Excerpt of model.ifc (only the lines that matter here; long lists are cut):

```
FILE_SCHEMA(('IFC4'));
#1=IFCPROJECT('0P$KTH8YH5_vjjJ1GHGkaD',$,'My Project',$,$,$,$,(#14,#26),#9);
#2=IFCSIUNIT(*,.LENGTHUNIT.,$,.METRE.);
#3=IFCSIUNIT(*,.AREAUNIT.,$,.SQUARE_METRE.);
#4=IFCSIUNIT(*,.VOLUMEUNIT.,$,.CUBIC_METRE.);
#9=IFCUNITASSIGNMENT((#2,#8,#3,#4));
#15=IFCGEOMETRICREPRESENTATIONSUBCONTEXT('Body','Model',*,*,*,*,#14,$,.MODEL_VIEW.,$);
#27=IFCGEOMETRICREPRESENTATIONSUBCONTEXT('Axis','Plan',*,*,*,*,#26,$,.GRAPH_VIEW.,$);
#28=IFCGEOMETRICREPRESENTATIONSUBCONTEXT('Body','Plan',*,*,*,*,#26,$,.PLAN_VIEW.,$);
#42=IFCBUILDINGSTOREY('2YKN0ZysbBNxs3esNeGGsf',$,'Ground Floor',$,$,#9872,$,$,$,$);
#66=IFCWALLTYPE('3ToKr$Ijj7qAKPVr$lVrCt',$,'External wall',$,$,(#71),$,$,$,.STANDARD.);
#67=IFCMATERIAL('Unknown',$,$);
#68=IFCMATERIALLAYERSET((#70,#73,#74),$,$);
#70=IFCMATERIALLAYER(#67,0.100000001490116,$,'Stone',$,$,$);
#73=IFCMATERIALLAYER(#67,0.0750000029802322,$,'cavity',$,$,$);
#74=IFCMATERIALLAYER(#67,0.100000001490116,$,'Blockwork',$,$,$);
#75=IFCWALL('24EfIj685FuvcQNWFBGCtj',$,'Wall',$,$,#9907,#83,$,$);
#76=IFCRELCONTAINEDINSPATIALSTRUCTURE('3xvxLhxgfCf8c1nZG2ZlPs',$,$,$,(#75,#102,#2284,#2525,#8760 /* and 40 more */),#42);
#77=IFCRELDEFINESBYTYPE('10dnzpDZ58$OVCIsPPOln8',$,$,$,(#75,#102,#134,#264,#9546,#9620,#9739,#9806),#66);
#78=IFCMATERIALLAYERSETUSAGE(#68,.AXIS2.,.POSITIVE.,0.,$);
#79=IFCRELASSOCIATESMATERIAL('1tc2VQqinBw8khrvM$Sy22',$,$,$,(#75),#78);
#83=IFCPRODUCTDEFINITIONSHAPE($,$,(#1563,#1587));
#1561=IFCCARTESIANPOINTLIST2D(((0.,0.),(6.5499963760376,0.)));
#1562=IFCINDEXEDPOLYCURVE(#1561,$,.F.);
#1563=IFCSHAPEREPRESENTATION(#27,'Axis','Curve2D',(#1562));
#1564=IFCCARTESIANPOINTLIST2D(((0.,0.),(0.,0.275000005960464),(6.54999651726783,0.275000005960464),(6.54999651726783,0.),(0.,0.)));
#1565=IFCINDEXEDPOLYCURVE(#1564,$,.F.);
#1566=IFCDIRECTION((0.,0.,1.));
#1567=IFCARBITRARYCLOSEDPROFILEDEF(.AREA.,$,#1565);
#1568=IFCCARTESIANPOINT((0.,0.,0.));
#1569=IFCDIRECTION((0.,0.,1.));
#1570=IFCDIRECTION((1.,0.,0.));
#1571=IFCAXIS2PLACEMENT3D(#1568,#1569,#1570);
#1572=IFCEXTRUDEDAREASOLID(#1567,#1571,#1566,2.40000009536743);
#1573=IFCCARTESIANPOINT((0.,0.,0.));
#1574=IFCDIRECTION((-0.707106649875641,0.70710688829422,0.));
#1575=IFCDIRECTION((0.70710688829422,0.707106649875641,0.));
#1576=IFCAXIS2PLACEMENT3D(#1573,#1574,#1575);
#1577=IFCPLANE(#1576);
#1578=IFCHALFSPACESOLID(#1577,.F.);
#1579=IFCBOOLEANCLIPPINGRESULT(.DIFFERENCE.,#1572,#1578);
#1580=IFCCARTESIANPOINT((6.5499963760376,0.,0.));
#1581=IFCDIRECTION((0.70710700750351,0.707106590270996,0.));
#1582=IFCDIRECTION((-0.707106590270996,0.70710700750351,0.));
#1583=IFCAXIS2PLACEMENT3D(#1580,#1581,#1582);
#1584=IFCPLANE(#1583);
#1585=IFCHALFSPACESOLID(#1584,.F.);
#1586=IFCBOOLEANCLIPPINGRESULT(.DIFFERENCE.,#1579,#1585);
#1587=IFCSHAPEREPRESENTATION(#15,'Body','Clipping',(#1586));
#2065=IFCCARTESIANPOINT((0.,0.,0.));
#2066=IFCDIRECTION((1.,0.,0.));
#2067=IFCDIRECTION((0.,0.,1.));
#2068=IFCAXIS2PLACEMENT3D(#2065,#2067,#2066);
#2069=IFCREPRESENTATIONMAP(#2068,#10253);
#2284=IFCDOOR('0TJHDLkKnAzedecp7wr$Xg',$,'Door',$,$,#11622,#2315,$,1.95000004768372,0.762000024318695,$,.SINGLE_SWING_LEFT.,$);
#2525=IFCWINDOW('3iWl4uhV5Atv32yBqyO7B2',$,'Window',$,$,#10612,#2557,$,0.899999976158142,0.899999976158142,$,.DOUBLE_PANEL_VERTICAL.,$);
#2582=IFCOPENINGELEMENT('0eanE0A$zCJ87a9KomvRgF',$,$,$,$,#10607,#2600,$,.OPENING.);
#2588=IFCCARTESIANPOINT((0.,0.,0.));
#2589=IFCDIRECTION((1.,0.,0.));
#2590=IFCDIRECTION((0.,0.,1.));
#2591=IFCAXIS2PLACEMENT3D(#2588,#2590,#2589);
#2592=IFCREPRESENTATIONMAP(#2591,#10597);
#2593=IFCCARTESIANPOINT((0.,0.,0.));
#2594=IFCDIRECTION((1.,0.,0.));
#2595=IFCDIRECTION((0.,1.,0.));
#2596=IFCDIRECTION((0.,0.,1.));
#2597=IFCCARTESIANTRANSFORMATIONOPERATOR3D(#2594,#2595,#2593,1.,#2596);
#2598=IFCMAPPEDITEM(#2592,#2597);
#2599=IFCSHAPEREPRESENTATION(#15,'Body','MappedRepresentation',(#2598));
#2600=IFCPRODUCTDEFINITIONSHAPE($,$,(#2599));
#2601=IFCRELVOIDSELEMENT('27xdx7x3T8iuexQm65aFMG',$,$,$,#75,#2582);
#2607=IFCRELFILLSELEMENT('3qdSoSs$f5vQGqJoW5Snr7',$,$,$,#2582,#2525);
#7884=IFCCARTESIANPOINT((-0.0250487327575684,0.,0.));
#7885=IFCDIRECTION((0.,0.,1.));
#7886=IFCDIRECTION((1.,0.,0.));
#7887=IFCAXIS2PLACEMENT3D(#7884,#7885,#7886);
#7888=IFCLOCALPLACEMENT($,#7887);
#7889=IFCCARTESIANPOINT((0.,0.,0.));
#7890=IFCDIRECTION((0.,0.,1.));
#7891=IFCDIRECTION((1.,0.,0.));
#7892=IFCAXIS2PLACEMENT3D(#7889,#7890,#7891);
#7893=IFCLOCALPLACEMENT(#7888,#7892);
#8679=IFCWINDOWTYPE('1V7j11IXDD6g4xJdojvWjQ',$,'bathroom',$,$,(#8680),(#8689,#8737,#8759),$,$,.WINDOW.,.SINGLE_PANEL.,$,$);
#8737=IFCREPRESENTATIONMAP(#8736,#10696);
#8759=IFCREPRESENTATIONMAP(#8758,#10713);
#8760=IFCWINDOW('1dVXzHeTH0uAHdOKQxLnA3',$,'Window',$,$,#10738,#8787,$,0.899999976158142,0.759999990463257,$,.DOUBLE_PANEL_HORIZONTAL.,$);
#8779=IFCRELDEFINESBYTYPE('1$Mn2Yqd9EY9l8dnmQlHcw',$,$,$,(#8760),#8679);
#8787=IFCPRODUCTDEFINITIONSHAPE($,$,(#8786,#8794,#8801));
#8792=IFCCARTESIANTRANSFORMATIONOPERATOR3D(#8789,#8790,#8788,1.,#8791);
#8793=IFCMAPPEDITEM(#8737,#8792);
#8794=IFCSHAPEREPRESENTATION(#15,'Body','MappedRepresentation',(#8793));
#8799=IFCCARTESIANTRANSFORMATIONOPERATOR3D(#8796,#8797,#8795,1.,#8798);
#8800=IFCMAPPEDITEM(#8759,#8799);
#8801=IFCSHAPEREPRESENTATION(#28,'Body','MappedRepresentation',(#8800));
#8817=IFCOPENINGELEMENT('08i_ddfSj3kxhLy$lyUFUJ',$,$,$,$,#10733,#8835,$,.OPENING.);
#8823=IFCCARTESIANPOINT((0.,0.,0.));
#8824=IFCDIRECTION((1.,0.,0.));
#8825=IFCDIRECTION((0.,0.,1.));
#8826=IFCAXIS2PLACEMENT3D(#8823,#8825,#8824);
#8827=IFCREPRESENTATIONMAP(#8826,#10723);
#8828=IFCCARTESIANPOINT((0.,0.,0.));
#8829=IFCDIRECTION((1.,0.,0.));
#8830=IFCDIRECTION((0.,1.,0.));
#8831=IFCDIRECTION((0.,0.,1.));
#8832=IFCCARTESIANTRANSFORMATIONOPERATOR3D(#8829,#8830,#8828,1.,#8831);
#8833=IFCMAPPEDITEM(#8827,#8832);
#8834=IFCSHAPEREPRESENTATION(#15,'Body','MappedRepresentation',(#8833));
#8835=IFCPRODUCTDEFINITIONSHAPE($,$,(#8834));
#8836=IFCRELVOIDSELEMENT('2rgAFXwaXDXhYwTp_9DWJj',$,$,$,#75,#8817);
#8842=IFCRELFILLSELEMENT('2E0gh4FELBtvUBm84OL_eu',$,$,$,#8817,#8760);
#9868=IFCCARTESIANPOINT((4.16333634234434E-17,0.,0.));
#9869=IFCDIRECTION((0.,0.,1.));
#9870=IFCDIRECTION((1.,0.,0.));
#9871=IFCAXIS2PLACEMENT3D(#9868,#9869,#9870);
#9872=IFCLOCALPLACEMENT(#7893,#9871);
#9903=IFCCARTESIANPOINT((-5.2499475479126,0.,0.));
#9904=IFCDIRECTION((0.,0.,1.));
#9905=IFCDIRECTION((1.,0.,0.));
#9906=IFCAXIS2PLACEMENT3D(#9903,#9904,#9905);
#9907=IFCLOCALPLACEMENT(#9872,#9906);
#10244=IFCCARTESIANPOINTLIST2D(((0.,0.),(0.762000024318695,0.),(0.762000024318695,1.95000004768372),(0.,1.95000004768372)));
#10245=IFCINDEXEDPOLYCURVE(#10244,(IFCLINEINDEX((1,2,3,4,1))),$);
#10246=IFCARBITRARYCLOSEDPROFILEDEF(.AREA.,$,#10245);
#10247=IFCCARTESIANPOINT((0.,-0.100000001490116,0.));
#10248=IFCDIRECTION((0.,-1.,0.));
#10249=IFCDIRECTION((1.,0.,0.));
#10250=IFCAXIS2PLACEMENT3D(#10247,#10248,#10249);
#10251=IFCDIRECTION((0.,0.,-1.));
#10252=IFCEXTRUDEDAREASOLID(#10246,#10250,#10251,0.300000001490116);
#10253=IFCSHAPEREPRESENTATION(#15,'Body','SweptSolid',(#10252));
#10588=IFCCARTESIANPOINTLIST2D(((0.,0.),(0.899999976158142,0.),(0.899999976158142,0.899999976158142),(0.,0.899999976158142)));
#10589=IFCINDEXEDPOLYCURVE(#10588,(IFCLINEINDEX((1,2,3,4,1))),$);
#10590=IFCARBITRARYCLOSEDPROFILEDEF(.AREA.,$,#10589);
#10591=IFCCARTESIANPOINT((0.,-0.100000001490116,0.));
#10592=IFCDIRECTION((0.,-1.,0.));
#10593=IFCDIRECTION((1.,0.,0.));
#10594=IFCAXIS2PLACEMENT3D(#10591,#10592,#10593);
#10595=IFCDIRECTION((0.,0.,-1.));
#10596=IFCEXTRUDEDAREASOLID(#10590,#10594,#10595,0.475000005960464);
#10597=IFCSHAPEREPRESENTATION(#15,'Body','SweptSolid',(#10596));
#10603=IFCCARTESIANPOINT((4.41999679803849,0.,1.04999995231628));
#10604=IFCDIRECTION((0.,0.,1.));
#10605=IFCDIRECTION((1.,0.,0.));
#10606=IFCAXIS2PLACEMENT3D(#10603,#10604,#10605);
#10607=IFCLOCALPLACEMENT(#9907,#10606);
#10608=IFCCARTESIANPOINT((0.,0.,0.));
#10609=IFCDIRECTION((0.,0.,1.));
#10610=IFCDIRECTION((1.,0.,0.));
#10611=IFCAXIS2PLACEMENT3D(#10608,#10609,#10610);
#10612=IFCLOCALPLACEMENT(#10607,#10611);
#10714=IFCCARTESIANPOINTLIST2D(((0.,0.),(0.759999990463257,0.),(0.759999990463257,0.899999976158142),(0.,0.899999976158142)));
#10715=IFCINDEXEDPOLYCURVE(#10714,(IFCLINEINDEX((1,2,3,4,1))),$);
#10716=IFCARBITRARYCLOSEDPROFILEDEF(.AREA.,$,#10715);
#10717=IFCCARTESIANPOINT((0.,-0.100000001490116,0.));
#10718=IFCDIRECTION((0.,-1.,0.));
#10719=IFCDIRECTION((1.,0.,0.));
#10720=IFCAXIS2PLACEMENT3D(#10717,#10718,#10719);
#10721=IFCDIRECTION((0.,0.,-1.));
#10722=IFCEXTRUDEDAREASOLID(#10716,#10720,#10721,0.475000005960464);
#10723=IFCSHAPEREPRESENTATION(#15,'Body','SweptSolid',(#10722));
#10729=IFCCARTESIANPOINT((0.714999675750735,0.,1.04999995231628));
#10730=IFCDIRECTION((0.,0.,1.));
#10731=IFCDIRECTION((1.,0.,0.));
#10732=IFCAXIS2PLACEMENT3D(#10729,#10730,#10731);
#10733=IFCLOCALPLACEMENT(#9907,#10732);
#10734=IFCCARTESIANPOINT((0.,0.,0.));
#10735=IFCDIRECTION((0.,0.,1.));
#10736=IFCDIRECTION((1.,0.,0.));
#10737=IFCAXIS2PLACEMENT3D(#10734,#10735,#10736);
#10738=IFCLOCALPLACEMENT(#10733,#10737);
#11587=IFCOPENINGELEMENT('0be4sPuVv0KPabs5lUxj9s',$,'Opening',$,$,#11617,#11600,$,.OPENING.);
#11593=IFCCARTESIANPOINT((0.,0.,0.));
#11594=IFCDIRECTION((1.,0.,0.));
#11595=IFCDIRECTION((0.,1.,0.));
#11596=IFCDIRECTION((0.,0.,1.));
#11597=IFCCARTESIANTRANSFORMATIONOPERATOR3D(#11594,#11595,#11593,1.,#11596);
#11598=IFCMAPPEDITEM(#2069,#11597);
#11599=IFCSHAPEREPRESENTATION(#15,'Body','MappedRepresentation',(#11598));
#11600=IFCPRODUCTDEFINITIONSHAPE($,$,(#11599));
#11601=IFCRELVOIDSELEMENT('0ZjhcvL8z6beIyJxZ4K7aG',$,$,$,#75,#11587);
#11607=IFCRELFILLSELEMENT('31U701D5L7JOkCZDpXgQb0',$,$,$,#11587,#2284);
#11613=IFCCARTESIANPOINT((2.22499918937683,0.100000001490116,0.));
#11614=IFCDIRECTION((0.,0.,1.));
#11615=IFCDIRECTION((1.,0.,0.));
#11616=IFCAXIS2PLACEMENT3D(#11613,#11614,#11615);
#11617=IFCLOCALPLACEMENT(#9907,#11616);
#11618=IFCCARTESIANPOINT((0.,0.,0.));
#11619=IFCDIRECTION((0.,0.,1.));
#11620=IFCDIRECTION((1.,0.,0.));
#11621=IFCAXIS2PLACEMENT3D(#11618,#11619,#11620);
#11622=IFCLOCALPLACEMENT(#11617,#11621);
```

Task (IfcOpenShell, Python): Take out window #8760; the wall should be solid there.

```python
import ifcopenshell
import ifcopenshell.api.feature
import ifcopenshell.api.root
import ifcopenshell.geom
import ifcopenshell.util.shape

model = ifcopenshell.open("model.ifc")
settings = ifcopenshell.geom.settings()


def volume(element):
    """Net volume in cubic metres, openings subtracted."""
    shape = ifcopenshell.geom.create_shape(settings, element)
    return ifcopenshell.util.shape.get_volume(shape.geometry)


window = model.by_id(8760)
opening = window.FillsVoids[0].RelatingOpeningElement
wall = opening.VoidsElements[0].RelatingBuildingElement
before = volume(wall)

ifcopenshell.api.root.remove_product(model, product=window)
ifcopenshell.api.feature.remove_feature(model, feature=opening)

after = volume(wall)

print(f"wall volume {before:.3f} -> {after:.3f} m3")

model.write("model-out.ifc")
```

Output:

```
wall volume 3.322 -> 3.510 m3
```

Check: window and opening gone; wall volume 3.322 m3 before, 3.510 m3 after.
